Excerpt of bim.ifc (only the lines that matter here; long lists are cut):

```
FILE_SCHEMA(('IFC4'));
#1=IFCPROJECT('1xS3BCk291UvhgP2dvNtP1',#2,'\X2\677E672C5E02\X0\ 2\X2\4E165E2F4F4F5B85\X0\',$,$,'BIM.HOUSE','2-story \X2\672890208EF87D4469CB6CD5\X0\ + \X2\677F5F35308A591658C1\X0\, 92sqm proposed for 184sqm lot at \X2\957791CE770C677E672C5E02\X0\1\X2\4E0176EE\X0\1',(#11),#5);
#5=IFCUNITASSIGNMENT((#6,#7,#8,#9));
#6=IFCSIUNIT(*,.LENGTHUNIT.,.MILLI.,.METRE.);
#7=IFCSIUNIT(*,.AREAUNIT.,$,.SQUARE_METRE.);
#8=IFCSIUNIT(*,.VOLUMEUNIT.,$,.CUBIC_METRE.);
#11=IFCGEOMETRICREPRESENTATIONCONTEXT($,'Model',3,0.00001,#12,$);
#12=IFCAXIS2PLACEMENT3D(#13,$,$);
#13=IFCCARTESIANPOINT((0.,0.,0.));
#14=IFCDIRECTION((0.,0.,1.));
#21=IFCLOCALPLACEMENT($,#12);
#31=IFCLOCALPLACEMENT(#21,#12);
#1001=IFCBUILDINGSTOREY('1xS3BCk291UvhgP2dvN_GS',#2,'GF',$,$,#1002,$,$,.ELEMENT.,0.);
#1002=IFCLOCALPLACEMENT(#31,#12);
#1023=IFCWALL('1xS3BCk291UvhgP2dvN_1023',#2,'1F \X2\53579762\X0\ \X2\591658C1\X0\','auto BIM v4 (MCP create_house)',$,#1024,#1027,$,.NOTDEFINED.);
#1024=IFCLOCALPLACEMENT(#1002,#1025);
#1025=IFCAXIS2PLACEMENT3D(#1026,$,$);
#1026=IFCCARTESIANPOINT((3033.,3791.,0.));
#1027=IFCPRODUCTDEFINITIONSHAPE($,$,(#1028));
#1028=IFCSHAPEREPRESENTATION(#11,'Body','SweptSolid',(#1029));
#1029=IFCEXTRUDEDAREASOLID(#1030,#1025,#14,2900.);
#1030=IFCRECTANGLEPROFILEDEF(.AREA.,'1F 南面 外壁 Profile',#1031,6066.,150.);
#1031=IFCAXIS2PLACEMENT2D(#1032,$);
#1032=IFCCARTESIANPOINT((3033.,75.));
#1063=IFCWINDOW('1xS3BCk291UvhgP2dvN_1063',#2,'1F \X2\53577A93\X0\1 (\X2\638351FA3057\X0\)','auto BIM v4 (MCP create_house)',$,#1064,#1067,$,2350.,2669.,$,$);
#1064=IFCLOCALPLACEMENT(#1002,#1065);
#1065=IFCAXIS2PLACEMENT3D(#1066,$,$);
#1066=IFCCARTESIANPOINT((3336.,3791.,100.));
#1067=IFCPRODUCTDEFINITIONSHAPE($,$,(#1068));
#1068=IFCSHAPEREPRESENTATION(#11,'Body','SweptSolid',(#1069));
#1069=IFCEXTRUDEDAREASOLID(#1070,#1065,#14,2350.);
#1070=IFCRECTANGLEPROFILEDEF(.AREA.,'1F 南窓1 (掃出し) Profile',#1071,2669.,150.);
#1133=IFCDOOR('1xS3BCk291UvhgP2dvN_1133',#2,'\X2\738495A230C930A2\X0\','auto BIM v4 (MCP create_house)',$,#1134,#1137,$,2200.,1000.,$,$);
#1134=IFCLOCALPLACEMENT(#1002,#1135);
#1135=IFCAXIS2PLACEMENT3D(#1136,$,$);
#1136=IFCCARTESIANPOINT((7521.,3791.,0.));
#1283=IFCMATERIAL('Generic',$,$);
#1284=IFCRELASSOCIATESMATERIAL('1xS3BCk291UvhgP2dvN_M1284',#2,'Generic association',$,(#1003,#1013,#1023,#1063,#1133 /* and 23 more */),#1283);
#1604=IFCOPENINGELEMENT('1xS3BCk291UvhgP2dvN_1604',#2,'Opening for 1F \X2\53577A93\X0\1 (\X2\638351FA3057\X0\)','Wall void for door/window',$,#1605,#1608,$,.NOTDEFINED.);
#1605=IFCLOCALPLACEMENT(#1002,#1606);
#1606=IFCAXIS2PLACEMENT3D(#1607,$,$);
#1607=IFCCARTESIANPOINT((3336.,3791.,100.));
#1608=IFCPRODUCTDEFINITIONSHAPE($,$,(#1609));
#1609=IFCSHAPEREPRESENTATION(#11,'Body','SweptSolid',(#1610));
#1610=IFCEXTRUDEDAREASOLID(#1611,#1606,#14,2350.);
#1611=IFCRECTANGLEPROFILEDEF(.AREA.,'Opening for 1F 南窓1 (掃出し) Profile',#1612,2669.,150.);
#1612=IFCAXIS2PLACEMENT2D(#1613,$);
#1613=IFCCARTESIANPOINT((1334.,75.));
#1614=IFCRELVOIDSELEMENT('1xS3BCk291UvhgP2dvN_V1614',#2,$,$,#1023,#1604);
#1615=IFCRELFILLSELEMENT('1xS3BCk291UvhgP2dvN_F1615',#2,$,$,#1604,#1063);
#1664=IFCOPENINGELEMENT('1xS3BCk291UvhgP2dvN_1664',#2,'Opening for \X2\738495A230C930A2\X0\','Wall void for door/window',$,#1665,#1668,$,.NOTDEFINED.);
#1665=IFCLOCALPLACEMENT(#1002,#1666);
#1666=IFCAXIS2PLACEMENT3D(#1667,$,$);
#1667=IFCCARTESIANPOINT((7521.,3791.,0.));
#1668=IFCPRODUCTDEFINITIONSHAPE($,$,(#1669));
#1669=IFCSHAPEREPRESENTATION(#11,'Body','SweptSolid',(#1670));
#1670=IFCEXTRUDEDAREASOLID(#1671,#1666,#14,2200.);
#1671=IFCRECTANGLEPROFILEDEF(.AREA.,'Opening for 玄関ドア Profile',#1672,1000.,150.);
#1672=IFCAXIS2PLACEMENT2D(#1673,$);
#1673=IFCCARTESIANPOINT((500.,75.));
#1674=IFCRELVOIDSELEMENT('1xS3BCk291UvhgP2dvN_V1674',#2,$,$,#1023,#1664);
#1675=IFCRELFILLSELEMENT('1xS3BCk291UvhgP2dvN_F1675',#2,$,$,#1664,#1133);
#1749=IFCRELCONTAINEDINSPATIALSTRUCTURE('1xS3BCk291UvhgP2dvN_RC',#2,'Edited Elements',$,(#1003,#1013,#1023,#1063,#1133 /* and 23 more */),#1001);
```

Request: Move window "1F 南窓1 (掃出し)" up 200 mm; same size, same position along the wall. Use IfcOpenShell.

```python
import numpy as np
import ifcopenshell
import ifcopenshell.api.geometry
import ifcopenshell.util.placement
import ifcopenshell.util.unit

model = ifcopenshell.open("bim.ifc")
unit_scale = ifcopenshell.util.unit.calculate_unit_scale(model)

window = model.by_guid("1xS3BCk291UvhgP2dvN_1063")
opening = window.FillsVoids[0].RelatingOpeningElement
dz = 0.2 / unit_scale

shift = np.array([0.0, 0.0, dz])
# The window is not placed relative to its opening, so move both.
for product in (opening, window):
    matrix = ifcopenshell.util.placement.get_local_placement(product.ObjectPlacement)
    matrix[:3, 3] += shift
    ifcopenshell.api.geometry.edit_object_placement(model, product=product, matrix=matrix, is_si=False)

print(f"moved by {dz * unit_scale:+.3f} m")

model.write("bim_rev.ifc")
```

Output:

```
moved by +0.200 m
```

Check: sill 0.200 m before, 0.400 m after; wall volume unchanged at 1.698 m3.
